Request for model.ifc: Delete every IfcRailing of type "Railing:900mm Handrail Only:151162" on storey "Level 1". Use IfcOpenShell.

First a look at what the model holds.

```python
import ifcopenshell
import ifcopenshell.util.element

model = ifcopenshell.open("model.ifc")
print(model.schema)
storey = next(s for s in model.by_type("IfcBuildingStorey") if s.Name == "Level 1")
railings = [e for e in ifcopenshell.util.element.get_decomposition(storey) if e.is_a("IfcRailing")]
seen = {}
for e in railings:
    element_type = ifcopenshell.util.element.get_type(e)
    name = element_type.Name if element_type not in (None, e) else None
    seen[name] = seen.get(name, 0) + 1
for name, count in sorted(seen.items(), key=str):
    print(count, "x", name)
```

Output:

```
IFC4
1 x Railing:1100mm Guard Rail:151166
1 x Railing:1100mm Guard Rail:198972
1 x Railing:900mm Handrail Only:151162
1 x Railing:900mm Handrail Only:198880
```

```python
import ifcopenshell
import ifcopenshell.api.root
import ifcopenshell.util.element

model = ifcopenshell.open("model.ifc")

storey = next(s for s in model.by_type("IfcBuildingStorey") if s.Name == "Level 1")
railings = [e for e in ifcopenshell.util.element.get_decomposition(storey) if e.is_a("IfcRailing")]
targets = [e for e in railings if (t := ifcopenshell.util.element.get_type(e)) not in (None, e) and t.Name == "Railing:900mm Handrail Only:151162"]

for e in targets:
    ifcopenshell.api.root.remove_product(model, product=e)
print(len(targets), "removed")

model.write("model_rev.ifc")
```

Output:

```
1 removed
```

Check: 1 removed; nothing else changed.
